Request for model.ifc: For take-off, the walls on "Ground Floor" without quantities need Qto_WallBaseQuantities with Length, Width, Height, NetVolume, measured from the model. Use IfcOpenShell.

First a look at what the model holds.

```python
import ifcopenshell
import ifcopenshell.util.element
import ifcopenshell.util.unit

model = ifcopenshell.open("model.ifc")
print(model.schema)
for unit_type in ("LENGTHUNIT", "AREAUNIT", "VOLUMEUNIT"):
    print(unit_type, ifcopenshell.util.unit.calculate_unit_scale(model, unit_type))
storey = next(s for s in model.by_type("IfcBuildingStorey") if s.Name == "Ground Floor")
walls = [e for e in ifcopenshell.util.element.get_decomposition(storey) if e.is_a("IfcWall")]
for e in sorted(walls, key=lambda e: e.id()):
    print(e.id(), e.is_a(), e.Name, list(ifcopenshell.util.element.get_psets(e, qtos_only=True)), sep=" | ")
```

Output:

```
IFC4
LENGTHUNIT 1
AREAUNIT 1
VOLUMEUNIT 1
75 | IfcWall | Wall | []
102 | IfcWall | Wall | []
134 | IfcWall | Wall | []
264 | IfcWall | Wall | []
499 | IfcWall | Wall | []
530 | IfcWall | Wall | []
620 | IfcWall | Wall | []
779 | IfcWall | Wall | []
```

```python
import ifcopenshell
import ifcopenshell.api.pset
import ifcopenshell.geom
import ifcopenshell.util.element
import ifcopenshell.util.shape
import ifcopenshell.util.unit

model = ifcopenshell.open("model.ifc")
unit_scale = ifcopenshell.util.unit.calculate_unit_scale(model)
volume_scale = ifcopenshell.util.unit.calculate_unit_scale(model, "VOLUMEUNIT")
settings = ifcopenshell.geom.settings()

storey = next(s for s in model.by_type("IfcBuildingStorey") if s.Name == "Ground Floor")
walls = [e for e in ifcopenshell.util.element.get_decomposition(storey) if e.is_a("IfcWall")]

for e in sorted(walls, key=lambda e: e.id()):
    if ifcopenshell.util.element.get_psets(e, qtos_only=True, should_inherit=False):
        continue
    # Geometry comes back in metres, in the element's own axes.
    shape = ifcopenshell.geom.create_shape(settings, e)
    values = {
        "Length": ifcopenshell.util.shape.get_x(shape.geometry) / unit_scale,
        "Width": ifcopenshell.util.shape.get_y(shape.geometry) / unit_scale,
        "Height": ifcopenshell.util.shape.get_z(shape.geometry) / unit_scale,
        "NetVolume": ifcopenshell.util.shape.get_volume(shape.geometry) / volume_scale,
    }
    qto = ifcopenshell.api.pset.add_qto(model, product=e, name="Qto_WallBaseQuantities")
    ifcopenshell.api.pset.edit_qto(model, qto=qto, properties=values)
    print(e.id(), {k: round(v, 3) for k, v in values.items()})

model.write("model-out.ifc")
```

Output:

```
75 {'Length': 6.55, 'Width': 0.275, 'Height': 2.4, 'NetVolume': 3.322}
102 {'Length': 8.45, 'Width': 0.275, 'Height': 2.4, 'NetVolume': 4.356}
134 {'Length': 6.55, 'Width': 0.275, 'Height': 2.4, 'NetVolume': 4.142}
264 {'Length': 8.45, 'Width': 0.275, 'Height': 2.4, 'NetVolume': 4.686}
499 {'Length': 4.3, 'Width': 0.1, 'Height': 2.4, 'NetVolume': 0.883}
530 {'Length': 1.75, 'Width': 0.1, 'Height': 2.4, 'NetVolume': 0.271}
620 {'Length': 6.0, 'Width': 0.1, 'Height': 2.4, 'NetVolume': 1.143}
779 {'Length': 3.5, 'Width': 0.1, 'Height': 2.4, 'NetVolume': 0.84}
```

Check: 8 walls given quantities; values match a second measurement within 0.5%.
